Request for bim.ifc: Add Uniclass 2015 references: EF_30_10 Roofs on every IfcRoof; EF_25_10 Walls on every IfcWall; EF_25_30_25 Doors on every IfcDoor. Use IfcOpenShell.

First a look at what the model holds.

```python
import ifcopenshell

model = ifcopenshell.open("bim.ifc")
print(model.schema)
print("classifications:", [c.Name for c in model.by_type("IfcClassification")])
for ifc_class in ("IfcDoor", "IfcRoof", "IfcStair", "IfcWall", "IfcWindow"):
    print(ifc_class, len(model.by_type(ifc_class)))
```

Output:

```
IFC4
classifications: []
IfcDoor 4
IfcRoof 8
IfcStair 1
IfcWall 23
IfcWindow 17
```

```python
import ifcopenshell
import ifcopenshell.api.classification

model = ifcopenshell.open("bim.ifc")

system = ifcopenshell.api.classification.add_classification(model, classification="Uniclass 2015")

codes = {
    "IfcRoof": ("EF_30_10", "Roofs"),
    "IfcWall": ("EF_25_10", "Walls"),
    "IfcDoor": ("EF_25_30_25", "Doors"),
}
for ifc_class, (code, name) in codes.items():
    products = model.by_type(ifc_class)
    ifcopenshell.api.classification.add_reference(
        model, products=products, classification=system, identification=code, name=name
    )
    print(code, len(products))

model.write("bim-out.ifc")
```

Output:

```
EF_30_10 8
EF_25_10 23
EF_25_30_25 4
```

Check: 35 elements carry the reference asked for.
